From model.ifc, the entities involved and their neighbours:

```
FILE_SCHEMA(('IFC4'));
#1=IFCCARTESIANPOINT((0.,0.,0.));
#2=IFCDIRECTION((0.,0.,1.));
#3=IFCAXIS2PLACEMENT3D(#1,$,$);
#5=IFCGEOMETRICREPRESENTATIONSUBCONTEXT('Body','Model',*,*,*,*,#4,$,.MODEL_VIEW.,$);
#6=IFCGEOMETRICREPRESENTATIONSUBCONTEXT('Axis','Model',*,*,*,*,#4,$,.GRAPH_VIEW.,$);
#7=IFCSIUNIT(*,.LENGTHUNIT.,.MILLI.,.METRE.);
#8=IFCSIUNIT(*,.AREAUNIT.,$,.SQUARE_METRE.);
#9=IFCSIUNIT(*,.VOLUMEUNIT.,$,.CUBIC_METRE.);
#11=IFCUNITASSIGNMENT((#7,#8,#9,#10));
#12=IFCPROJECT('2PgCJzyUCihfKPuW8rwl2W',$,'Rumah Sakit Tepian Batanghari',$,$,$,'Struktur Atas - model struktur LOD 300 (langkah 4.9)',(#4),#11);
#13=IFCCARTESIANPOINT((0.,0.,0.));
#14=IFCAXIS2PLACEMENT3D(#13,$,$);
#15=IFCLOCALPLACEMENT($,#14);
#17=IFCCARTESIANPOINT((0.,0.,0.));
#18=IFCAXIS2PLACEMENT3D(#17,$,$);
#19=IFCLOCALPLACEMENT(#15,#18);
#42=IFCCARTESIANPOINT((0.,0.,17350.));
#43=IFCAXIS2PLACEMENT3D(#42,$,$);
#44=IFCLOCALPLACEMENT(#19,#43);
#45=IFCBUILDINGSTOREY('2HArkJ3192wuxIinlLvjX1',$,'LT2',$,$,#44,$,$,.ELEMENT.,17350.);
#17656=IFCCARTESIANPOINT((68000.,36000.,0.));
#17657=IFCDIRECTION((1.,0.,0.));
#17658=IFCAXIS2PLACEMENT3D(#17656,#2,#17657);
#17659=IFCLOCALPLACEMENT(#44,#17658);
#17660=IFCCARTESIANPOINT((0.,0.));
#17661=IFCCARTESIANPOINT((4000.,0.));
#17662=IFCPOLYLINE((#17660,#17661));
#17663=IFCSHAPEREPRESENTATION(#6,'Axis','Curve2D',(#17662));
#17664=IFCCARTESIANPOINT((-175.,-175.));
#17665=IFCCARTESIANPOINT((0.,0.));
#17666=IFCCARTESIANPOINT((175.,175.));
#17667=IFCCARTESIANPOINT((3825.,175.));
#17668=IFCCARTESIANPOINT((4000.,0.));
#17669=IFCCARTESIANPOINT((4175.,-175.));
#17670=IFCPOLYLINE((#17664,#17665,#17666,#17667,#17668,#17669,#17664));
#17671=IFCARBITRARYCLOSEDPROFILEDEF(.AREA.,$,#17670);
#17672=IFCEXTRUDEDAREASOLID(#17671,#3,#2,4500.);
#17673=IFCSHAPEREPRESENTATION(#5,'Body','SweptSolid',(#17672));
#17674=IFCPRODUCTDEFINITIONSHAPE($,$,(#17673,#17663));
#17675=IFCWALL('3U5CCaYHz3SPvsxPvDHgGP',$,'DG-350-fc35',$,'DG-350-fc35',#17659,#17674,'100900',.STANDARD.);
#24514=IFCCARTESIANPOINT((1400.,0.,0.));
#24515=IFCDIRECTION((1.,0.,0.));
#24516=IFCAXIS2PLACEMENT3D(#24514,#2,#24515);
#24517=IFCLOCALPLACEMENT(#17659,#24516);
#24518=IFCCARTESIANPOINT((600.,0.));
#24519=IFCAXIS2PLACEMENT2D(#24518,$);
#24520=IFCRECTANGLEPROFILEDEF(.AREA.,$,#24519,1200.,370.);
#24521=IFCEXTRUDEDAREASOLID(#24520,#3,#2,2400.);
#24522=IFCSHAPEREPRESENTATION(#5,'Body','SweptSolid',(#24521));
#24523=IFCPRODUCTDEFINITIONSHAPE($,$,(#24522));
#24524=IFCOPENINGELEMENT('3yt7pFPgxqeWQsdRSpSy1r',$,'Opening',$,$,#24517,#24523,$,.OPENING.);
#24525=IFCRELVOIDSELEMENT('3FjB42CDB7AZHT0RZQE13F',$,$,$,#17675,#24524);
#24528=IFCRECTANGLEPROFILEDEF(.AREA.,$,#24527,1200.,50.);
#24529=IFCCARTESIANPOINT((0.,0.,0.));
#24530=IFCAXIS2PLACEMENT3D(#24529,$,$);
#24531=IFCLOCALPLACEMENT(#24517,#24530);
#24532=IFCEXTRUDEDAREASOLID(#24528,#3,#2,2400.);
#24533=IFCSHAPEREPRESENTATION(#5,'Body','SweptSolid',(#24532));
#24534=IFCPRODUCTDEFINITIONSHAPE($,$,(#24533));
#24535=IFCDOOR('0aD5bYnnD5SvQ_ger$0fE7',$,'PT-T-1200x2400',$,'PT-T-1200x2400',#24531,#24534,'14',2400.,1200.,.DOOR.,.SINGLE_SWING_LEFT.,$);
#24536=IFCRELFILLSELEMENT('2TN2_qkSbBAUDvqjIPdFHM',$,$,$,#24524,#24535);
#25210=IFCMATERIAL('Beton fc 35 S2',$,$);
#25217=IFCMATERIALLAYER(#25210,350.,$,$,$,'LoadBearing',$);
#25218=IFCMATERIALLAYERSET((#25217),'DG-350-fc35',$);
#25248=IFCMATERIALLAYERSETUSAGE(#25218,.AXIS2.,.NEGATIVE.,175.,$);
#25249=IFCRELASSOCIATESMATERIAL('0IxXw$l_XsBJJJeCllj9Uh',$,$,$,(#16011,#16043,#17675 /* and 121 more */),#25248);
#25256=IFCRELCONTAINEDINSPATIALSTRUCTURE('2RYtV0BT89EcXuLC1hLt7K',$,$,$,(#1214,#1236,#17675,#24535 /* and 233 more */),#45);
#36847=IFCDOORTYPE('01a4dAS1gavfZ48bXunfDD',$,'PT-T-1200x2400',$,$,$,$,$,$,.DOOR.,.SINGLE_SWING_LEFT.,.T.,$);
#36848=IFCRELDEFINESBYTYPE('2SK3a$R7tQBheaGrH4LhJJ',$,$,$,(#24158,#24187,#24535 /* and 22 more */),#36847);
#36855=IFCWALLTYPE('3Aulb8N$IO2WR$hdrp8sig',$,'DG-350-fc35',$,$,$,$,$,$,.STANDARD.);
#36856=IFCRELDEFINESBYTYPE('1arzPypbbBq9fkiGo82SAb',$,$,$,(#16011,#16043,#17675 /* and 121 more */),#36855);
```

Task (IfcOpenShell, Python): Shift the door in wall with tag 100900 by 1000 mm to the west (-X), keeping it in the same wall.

```python
import ifcopenshell
import ifcopenshell.api.geometry
import ifcopenshell.util.placement

model = ifcopenshell.open("model.ifc")

door = model.by_id(24535)
opening = door.FillsVoids[0].RelatingOpeningElement
wall = opening.VoidsElements[0].RelatingBuildingElement

wall_matrix = ifcopenshell.util.placement.get_local_placement(wall.ObjectPlacement)
shift = wall_matrix[:3, 0] * -1000.0
before = ifcopenshell.util.placement.get_local_placement(door.ObjectPlacement)[:3, 3].copy()

# The door is placed relative to its opening, so it follows when the opening moves.
matrix = ifcopenshell.util.placement.get_local_placement(opening.ObjectPlacement)
matrix[:3, 3] += shift
ifcopenshell.api.geometry.edit_object_placement(
    model, product=opening, matrix=matrix, is_si=False, should_transform_children=True
)

after = ifcopenshell.util.placement.get_local_placement(door.ObjectPlacement)[:3, 3]
print("door moved by", (after - before).round(3) + 0.0)

model.write("model_v2.ifc")
```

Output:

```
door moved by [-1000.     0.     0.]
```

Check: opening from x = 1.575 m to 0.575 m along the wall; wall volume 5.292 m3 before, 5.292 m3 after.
